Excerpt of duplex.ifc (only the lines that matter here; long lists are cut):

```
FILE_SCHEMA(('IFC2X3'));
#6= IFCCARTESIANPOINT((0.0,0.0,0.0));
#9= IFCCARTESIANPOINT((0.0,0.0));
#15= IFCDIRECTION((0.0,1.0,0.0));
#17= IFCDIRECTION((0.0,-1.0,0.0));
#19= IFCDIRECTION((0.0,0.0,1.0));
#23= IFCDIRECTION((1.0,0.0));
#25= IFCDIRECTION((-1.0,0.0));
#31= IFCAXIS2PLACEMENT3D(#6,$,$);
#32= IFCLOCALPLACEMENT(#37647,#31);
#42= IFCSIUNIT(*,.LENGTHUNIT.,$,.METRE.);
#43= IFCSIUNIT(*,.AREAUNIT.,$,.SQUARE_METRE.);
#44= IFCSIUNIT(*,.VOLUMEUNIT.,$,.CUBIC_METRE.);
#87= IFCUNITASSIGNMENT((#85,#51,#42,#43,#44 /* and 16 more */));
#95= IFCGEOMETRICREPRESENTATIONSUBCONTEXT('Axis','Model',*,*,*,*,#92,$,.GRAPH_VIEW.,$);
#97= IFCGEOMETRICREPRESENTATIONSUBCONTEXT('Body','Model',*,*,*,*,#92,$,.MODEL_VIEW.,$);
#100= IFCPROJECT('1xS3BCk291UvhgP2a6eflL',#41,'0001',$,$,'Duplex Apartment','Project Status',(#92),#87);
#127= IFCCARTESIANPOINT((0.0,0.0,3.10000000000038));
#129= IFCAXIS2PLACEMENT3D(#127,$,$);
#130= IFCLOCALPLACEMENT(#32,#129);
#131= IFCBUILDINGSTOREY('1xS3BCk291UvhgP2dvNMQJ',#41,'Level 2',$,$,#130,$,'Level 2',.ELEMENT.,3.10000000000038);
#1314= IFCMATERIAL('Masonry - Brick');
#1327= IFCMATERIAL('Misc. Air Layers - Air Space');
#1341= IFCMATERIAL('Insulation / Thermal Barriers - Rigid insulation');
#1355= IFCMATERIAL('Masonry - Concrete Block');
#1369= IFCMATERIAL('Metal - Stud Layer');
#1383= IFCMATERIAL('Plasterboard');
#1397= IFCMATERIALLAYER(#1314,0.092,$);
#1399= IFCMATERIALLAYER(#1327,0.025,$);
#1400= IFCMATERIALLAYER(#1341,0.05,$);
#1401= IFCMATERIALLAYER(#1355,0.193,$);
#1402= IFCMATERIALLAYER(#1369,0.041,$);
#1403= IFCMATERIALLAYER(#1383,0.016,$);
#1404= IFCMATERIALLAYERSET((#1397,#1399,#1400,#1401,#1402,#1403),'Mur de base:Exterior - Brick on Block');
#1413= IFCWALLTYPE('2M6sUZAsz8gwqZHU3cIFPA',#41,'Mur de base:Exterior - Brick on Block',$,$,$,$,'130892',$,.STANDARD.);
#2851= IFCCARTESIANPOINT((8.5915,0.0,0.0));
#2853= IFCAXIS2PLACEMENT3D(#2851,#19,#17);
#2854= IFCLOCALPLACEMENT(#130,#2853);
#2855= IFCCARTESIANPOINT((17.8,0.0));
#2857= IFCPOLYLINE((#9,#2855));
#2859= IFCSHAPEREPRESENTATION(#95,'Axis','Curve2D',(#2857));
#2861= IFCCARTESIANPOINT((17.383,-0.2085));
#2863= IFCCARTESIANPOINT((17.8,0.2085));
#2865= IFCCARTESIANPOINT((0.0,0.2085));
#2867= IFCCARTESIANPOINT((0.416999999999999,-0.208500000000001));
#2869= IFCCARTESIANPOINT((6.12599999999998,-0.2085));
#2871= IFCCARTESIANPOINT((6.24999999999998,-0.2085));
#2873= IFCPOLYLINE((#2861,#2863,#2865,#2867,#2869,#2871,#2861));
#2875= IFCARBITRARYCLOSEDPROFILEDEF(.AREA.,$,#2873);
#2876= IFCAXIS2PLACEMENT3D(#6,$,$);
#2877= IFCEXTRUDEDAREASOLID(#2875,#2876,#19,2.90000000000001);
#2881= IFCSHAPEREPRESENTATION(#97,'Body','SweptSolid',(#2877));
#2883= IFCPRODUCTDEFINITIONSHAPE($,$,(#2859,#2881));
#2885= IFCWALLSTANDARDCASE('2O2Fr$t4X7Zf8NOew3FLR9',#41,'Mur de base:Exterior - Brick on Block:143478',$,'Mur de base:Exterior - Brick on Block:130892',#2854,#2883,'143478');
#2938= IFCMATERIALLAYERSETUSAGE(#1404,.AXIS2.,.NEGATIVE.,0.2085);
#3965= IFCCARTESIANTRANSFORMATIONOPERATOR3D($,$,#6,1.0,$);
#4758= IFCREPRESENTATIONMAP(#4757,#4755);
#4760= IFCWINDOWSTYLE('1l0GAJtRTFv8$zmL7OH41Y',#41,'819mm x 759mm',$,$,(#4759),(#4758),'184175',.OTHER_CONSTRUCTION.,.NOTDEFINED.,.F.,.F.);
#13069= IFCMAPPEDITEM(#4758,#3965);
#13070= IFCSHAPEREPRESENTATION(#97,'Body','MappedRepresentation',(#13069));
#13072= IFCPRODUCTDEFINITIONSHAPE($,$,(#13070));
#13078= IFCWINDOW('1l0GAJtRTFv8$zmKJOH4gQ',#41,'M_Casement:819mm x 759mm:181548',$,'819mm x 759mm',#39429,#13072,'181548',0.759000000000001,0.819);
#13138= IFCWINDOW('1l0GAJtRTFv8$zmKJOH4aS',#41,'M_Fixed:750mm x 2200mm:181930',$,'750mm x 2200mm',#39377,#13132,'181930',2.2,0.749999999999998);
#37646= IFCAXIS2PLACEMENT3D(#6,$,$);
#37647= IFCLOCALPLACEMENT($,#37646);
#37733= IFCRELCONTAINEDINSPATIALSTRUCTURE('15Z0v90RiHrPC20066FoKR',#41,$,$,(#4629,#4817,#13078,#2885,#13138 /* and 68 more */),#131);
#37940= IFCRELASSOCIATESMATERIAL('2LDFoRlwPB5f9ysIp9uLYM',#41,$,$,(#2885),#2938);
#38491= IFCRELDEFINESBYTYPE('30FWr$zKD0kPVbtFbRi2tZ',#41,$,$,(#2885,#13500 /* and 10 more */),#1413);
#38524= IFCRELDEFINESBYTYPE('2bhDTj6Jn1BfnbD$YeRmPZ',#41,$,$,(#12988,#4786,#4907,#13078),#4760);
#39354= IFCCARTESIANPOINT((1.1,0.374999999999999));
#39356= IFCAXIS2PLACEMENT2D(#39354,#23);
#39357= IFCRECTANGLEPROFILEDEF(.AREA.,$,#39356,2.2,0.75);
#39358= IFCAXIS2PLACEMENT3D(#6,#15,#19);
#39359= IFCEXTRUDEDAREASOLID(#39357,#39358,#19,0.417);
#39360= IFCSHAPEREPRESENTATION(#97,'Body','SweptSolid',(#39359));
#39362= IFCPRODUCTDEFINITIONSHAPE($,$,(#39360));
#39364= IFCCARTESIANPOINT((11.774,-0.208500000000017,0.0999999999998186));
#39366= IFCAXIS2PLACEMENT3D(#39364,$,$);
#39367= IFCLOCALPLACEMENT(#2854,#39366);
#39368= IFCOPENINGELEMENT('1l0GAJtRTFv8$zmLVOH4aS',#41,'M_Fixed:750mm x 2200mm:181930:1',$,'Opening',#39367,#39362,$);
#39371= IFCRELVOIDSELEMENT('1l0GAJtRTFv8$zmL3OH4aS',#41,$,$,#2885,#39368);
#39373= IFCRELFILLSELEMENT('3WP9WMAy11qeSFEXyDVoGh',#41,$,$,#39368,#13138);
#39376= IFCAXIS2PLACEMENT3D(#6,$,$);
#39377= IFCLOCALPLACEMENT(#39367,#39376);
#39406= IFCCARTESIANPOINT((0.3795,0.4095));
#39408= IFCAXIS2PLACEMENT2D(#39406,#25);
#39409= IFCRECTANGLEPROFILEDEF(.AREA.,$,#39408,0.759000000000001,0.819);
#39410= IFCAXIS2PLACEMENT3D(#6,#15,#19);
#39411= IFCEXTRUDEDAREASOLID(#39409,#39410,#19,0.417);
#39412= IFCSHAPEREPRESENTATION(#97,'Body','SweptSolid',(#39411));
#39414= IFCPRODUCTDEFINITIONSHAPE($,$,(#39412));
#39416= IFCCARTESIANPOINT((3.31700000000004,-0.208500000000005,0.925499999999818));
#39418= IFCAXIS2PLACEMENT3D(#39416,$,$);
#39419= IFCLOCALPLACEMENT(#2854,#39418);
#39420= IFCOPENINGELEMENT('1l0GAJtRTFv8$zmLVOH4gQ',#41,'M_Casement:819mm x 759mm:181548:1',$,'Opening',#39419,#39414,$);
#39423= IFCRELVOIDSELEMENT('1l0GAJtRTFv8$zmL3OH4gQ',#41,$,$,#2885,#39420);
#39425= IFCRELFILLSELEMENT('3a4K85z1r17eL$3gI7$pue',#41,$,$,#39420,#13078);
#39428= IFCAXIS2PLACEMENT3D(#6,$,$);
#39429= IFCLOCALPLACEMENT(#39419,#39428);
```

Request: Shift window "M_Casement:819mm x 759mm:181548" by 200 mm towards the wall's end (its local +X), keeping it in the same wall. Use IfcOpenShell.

```python
import ifcopenshell
import ifcopenshell.api.geometry
import ifcopenshell.util.placement
import ifcopenshell.util.unit

model = ifcopenshell.open("duplex.ifc")
unit_scale = ifcopenshell.util.unit.calculate_unit_scale(model)

window = model.by_id(13078)
opening = window.FillsVoids[0].RelatingOpeningElement
wall = opening.VoidsElements[0].RelatingBuildingElement

wall_matrix = ifcopenshell.util.placement.get_local_placement(wall.ObjectPlacement)
shift = wall_matrix[:3, 0] * 0.2 / unit_scale
before = ifcopenshell.util.placement.get_local_placement(window.ObjectPlacement)[:3, 3].copy()

# The window is placed relative to its opening, so it follows when the opening moves.
matrix = ifcopenshell.util.placement.get_local_placement(opening.ObjectPlacement)
matrix[:3, 3] += shift
ifcopenshell.api.geometry.edit_object_placement(
    model, product=opening, matrix=matrix, is_si=False, should_transform_children=True
)

after = ifcopenshell.util.placement.get_local_placement(window.ObjectPlacement)[:3, 3]
print("window moved by", (after - before).round(3) + 0.0)

model.write("duplex_updated.ifc")
```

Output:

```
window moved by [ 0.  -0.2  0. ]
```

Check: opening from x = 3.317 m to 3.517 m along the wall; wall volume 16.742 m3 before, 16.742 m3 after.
